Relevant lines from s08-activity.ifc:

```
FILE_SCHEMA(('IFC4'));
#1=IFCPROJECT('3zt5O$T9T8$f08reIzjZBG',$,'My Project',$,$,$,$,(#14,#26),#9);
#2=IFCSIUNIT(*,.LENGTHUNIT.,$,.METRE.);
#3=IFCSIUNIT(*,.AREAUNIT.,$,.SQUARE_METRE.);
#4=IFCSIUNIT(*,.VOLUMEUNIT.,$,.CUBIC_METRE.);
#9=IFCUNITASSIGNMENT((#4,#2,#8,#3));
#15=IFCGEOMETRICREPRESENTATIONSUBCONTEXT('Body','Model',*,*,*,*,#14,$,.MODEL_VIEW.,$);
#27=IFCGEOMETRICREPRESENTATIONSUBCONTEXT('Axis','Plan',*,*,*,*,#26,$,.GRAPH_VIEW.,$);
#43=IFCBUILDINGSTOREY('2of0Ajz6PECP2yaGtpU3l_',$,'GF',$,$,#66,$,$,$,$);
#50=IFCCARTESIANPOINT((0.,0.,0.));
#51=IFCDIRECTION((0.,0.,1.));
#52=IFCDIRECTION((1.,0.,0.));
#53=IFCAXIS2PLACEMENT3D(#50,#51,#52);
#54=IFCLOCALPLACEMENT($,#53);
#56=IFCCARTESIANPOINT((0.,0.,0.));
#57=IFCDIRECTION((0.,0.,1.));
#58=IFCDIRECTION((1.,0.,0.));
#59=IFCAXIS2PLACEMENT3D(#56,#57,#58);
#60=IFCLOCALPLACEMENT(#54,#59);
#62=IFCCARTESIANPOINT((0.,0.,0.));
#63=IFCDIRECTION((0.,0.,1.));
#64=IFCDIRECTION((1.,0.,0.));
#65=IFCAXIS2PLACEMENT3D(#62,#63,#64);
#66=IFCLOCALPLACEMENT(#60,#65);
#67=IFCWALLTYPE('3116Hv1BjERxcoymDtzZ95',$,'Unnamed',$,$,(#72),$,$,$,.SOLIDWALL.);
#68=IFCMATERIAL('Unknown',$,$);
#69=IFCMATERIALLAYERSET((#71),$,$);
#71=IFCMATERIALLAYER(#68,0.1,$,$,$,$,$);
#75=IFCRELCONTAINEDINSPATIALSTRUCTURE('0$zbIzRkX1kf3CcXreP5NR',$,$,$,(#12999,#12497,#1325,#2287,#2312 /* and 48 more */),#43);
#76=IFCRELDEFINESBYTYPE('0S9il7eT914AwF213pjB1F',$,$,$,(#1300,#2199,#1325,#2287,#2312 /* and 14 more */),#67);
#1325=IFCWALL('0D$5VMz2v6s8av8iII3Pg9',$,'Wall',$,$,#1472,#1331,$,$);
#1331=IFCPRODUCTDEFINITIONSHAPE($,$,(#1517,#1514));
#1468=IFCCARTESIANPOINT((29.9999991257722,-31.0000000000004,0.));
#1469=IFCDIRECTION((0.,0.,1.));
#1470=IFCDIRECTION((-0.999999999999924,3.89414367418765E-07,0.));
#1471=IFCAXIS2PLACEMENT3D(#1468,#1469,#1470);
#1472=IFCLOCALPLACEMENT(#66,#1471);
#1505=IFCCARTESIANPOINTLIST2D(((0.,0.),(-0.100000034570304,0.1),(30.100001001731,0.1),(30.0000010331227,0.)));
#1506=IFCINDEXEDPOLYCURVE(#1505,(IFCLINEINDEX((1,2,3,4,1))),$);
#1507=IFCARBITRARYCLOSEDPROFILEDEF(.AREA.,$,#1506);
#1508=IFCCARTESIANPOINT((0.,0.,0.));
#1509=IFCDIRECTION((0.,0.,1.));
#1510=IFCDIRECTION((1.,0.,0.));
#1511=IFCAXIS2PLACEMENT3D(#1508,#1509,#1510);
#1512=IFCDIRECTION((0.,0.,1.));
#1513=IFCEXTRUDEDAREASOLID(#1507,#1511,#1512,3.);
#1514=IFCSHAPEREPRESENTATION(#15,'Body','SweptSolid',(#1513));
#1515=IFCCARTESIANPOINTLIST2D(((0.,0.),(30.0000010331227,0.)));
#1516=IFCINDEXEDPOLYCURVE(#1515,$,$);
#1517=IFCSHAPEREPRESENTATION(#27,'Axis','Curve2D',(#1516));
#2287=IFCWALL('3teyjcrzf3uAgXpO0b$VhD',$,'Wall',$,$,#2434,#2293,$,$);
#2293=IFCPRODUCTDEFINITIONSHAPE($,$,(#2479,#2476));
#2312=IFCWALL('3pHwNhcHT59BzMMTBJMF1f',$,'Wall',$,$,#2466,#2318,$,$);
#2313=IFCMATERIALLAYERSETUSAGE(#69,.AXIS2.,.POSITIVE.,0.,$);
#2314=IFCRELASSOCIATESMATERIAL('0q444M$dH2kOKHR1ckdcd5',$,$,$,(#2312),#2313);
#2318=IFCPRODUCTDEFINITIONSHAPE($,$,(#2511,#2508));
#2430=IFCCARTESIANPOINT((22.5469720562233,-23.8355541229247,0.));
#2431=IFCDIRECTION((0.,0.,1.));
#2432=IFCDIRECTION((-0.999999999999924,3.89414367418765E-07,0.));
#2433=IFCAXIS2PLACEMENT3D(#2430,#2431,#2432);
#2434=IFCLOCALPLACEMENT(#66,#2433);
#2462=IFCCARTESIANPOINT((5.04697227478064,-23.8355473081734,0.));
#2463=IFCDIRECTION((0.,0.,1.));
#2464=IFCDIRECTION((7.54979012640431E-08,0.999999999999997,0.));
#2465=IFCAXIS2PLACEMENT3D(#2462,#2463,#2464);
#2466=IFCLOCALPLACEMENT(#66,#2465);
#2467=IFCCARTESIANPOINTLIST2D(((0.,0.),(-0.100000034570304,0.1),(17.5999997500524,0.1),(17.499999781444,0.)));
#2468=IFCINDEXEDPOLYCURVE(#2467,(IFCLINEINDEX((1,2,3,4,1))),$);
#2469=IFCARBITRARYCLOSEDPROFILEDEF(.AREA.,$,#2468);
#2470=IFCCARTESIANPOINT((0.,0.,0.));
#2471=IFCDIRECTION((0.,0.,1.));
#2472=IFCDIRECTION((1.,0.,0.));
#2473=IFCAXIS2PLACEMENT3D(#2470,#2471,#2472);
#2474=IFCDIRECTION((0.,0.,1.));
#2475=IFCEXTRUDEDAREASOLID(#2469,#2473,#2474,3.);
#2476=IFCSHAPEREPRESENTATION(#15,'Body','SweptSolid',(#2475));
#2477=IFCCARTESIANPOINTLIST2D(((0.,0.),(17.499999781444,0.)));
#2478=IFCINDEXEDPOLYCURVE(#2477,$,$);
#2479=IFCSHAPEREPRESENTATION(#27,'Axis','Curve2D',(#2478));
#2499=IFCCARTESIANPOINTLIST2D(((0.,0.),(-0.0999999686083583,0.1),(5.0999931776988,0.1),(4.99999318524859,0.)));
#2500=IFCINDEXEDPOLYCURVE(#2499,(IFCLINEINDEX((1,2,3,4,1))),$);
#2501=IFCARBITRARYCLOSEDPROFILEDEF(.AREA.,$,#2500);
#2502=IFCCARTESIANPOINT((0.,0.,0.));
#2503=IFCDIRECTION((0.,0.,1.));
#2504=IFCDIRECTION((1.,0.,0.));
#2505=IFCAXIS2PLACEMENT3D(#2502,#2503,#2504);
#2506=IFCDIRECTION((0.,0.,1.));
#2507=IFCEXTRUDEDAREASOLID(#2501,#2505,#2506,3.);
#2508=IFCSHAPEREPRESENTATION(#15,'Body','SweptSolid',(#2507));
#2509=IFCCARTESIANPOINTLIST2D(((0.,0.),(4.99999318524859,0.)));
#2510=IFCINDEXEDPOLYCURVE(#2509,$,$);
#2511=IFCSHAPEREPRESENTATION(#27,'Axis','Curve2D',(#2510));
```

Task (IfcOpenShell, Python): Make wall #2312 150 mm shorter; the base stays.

```python
import ifcopenshell
import ifcopenshell.geom
import ifcopenshell.util.representation
import ifcopenshell.util.shape

model = ifcopenshell.open("s08-activity.ifc")
settings = ifcopenshell.geom.settings()


def volume(element):
    """Net volume in cubic metres, openings subtracted."""
    shape = ifcopenshell.geom.create_shape(settings, element)
    return ifcopenshell.util.shape.get_volume(shape.geometry)


wall = model.by_id(2312)
before = volume(wall)

body = ifcopenshell.util.representation.get_representation(wall, "Model", "Body")
solid = body.Items[0]
old_height = solid.Depth
solid.Depth -= 0.15
after = volume(wall)

print(f"height {old_height:g} -> {solid.Depth:g}, volume {before:.3f} -> {after:.3f} m3")

model.write("s08-activity-out.ifc")
```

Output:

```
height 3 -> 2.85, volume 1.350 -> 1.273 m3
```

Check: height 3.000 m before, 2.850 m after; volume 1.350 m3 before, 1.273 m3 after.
